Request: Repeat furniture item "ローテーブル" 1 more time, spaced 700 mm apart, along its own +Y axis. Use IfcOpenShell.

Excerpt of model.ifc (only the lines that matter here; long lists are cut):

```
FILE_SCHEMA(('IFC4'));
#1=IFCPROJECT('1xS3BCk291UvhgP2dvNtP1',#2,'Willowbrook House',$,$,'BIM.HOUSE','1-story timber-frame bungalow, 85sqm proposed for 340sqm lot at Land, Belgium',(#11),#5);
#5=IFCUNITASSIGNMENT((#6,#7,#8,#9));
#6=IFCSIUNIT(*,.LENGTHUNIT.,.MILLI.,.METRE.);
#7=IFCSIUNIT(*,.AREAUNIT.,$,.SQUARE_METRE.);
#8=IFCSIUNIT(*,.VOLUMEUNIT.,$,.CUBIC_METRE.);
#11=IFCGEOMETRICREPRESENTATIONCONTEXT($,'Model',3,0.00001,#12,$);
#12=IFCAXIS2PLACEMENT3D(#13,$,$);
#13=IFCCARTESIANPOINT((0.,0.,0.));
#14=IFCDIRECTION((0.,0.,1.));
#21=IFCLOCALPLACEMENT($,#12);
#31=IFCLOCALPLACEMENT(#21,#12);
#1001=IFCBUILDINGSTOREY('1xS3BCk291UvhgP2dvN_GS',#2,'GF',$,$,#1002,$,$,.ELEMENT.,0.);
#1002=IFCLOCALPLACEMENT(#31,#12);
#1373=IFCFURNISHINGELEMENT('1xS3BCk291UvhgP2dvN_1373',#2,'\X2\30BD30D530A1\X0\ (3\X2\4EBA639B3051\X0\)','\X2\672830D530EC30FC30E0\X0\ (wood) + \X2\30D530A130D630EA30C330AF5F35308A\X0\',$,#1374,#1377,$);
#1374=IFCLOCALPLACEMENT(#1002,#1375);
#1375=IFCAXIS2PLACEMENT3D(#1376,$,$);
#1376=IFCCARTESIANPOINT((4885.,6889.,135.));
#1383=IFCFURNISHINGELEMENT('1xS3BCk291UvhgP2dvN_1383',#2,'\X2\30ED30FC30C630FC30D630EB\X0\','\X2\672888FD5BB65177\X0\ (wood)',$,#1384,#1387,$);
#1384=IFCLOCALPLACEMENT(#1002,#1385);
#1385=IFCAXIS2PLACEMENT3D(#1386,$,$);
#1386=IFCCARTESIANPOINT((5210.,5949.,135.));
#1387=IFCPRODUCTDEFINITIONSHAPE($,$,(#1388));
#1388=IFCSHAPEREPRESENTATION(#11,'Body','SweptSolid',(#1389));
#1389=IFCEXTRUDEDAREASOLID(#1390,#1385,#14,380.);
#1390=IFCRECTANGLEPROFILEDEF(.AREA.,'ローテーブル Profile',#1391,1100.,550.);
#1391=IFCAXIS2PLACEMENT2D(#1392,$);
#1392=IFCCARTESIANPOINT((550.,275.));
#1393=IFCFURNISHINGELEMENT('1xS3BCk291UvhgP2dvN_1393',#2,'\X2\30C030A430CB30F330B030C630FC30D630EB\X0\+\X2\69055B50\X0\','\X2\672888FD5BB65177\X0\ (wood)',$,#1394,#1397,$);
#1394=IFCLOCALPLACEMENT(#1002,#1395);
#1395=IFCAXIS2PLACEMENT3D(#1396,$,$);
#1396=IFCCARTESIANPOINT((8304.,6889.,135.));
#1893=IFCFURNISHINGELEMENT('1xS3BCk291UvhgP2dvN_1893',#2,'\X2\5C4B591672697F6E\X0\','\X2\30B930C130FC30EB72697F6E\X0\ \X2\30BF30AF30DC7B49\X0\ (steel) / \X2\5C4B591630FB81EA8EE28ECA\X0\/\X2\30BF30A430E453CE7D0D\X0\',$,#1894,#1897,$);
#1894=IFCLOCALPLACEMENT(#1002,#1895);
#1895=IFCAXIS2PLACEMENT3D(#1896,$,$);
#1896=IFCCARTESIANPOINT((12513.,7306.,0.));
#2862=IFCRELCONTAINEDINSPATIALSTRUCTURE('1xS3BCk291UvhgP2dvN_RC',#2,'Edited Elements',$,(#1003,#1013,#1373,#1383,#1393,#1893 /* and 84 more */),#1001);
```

```python
import ifcopenshell
import ifcopenshell.api.geometry
import ifcopenshell.api.root
import ifcopenshell.util.element
import ifcopenshell.util.placement

model = ifcopenshell.open("model.ifc")


def reuse_history(source, copy):
    """copy_class also copies each property set's owner history, people and application; keep the originals."""
    for rel in copy.IsDefinedBy:
        if rel.is_a("IfcRelDefinesByProperties") and (history := rel.RelatingPropertyDefinition.OwnerHistory):
            rel.RelatingPropertyDefinition.OwnerHistory = source.OwnerHistory
            ifcopenshell.util.element.remove_deep2(model, history)


source = model.by_id(1383)
base = ifcopenshell.util.placement.get_local_placement(source.ObjectPlacement)
step = base[:3, 1] * 700.0

for i in range(1, 2):
    copy = ifcopenshell.api.root.copy_class(model, product=source)
    copy.Representation = ifcopenshell.util.element.copy_deep(
        model, source.Representation, exclude=["IfcGeometricRepresentationContext", "IfcRepresentationMap"]
    )
    reuse_history(source, copy)
    matrix = base.copy()
    matrix[:3, 3] += i * step
    print("added at", matrix[:3, 3].round(3) + 0.0)
    ifcopenshell.api.geometry.edit_object_placement(model, product=copy, matrix=matrix, is_si=False)

model.write("model-out.ifc")
```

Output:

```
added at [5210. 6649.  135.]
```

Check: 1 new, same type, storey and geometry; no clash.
